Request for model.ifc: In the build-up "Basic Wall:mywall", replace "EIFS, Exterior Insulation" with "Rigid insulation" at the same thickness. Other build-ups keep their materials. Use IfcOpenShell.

First a look at what the model holds.

```python
import ifcopenshell
import ifcopenshell.util.element

model = ifcopenshell.open("model.ifc")
print(model.schema)
for layer_set in model.by_type("IfcMaterialLayerSet"):
    if layer_set.LayerSetName == "Basic Wall:mywall":
        for layer in layer_set.MaterialLayers:
            print(layer.id(), layer.Material and layer.Material.Name, layer.LayerThickness, sep=" | ")
        print(len(ifcopenshell.util.element.get_elements_by_material(model, layer_set)), "elements and types use it")
print(sorted(m.Name for m in model.by_type("IfcMaterial") if m.Name)[:60])
```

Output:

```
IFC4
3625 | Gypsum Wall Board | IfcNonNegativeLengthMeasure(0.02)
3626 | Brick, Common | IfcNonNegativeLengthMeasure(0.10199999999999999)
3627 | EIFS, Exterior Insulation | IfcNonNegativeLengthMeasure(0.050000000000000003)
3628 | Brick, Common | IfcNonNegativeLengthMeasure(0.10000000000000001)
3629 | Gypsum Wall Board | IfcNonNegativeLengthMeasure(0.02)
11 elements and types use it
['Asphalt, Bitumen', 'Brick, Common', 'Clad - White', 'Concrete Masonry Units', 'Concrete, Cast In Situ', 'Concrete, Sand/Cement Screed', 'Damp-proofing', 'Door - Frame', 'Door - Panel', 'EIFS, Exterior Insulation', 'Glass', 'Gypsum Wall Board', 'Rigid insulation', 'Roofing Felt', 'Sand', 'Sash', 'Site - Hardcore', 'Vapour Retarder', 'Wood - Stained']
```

```python
import ifcopenshell
import ifcopenshell.api.material

model = ifcopenshell.open("model.ifc")

layer_set = next(s for s in model.by_type("IfcMaterialLayerSet") if s.LayerSetName == "Basic Wall:mywall")
layer = next(l for l in layer_set.MaterialLayers if l.Material and l.Material.Name == "EIFS, Exterior Insulation")
material = next(m for m in model.by_type("IfcMaterial") if m.Name == "Rigid insulation")

# Point this one layer at the other material; renaming the old one would change it everywhere.
ifcopenshell.api.material.edit_layer(model, layer=layer, attributes={"Name": material.Name}, material=material)

print([l.Material.Name if l.Material else None for l in layer_set.MaterialLayers])

model.write("model-out.ifc")
```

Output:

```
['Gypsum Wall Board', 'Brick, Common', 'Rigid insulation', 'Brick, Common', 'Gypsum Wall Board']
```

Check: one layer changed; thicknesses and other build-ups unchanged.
